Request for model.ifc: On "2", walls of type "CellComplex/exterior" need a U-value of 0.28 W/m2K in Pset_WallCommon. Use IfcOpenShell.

First a look at what the model holds.

```python
import ifcopenshell
import ifcopenshell.util.element

model = ifcopenshell.open("model.ifc")
print(model.schema)
storey = next(s for s in model.by_type("IfcBuildingStorey") if s.Name == "2")
walls = [e for e in ifcopenshell.util.element.get_decomposition(storey) if e.is_a("IfcWall")]
seen = {}
for e in walls:
    element_type = ifcopenshell.util.element.get_type(e)
    key = (element_type.Name if element_type != e and element_type else None, ifcopenshell.util.element.get_pset(e, "Pset_WallCommon", "ThermalTransmittance"))
    seen[key] = seen.get(key, 0) + 1
for (name, value), count in sorted(seen.items(), key=str):
    print(count, "x", name, "|", value)
```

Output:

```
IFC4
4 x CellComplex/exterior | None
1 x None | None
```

```python
import ifcopenshell
import ifcopenshell.api.pset
import ifcopenshell.util.element

model = ifcopenshell.open("model.ifc")

storey = next(s for s in model.by_type("IfcBuildingStorey") if s.Name == "2")
walls = [e for e in ifcopenshell.util.element.get_decomposition(storey) if e.is_a("IfcWall")]

count = 0
for e in walls:
    element_type = ifcopenshell.util.element.get_type(e)
    if element_type in (None, e) or element_type.Name != "CellComplex/exterior":
        continue
    # add_pset returns the element's existing set when there is one.
    pset = ifcopenshell.api.pset.add_pset(model, product=e, name="Pset_WallCommon")
    ifcopenshell.api.pset.edit_pset(model, pset=pset, properties={"ThermalTransmittance": 0.28})
    count += 1

print(count, "walls updated")

model.write("model_rev.ifc")
```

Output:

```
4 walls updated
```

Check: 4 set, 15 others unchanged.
